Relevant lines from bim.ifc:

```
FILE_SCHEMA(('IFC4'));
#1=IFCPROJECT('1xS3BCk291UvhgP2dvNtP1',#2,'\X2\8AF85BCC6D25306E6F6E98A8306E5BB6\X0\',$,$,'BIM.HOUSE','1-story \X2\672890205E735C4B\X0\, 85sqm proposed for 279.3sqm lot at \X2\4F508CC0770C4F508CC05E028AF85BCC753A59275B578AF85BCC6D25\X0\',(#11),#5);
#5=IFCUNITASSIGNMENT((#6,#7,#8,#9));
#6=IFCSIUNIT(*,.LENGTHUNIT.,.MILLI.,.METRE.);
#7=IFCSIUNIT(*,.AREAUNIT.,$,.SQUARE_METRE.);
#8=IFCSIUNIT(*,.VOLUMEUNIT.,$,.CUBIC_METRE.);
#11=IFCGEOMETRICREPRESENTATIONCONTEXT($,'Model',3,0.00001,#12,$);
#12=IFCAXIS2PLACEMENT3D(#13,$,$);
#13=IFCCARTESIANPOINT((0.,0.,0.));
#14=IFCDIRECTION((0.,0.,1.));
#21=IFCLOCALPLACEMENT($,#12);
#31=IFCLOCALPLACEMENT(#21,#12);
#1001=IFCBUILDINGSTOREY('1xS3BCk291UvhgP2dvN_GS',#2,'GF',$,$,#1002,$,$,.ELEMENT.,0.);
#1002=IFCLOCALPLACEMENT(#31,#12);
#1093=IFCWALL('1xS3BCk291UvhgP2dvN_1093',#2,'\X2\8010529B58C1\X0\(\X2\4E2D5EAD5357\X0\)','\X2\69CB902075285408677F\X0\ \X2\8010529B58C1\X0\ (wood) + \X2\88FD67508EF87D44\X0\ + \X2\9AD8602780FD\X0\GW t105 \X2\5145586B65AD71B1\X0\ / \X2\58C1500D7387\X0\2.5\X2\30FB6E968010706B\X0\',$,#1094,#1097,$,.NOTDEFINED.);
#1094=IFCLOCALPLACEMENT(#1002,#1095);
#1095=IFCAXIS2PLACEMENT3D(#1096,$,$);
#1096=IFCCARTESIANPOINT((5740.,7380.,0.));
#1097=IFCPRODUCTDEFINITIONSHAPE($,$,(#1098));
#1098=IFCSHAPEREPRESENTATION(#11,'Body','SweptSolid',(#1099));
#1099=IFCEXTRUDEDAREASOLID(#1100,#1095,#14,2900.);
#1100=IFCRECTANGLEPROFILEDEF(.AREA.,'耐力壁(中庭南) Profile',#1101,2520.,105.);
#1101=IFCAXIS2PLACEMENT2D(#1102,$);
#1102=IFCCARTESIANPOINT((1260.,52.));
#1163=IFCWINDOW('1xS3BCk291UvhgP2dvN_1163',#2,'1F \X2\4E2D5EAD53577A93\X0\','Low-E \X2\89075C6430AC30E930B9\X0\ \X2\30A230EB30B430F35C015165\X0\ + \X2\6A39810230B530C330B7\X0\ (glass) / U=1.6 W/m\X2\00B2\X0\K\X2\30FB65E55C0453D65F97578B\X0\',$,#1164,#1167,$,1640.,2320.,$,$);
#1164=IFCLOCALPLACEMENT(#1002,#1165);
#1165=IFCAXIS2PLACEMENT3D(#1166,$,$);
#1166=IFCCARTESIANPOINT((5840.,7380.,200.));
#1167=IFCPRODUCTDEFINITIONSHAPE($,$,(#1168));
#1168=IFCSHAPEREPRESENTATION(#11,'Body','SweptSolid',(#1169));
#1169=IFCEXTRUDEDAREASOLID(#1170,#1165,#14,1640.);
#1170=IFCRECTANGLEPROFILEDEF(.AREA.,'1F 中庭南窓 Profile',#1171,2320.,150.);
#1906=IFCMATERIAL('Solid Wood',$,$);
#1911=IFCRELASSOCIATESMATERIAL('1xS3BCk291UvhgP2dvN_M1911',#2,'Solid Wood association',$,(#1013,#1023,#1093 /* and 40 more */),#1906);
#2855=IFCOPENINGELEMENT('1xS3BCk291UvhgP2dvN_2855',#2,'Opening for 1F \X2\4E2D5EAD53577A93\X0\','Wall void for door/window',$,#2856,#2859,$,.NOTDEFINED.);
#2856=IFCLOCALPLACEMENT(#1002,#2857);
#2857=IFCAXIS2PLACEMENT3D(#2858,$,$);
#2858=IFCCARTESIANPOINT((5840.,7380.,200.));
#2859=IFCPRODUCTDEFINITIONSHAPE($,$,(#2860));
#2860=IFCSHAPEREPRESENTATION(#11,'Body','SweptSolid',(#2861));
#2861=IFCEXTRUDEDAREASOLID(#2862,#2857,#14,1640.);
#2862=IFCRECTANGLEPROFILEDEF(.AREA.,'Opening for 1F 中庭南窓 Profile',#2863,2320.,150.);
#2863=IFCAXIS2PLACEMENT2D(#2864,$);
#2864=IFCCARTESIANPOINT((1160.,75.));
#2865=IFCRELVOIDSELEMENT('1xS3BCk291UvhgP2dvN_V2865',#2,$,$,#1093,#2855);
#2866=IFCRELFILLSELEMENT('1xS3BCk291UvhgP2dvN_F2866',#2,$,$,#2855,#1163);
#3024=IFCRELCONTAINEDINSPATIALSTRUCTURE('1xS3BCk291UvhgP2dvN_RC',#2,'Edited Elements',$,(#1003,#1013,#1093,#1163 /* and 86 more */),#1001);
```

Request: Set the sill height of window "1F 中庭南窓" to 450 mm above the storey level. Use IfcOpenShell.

```python
import numpy as np
import ifcopenshell
import ifcopenshell.api.geometry
import ifcopenshell.geom
import ifcopenshell.util.element
import ifcopenshell.util.placement
import ifcopenshell.util.shape
import ifcopenshell.util.unit

model = ifcopenshell.open("bim.ifc")
unit_scale = ifcopenshell.util.unit.calculate_unit_scale(model)

window = model.by_guid("1xS3BCk291UvhgP2dvN_1163")
opening = window.FillsVoids[0].RelatingOpeningElement
storey = ifcopenshell.util.element.get_container(window, ifc_class="IfcBuildingStorey")
level = ifcopenshell.util.placement.get_local_placement(storey.ObjectPlacement)[2, 3]

# The opening's origin need not be at the sill, so measure its lowest point.
shape = ifcopenshell.geom.create_shape(ifcopenshell.geom.settings(), opening)
bottom = ifcopenshell.util.shape.get_shape_bottom_elevation(shape, shape.geometry) / unit_scale
dz = level + 0.45 / unit_scale - bottom

shift = np.array([0.0, 0.0, dz])
# The window is not placed relative to its opening, so move both.
for product in (opening, window):
    matrix = ifcopenshell.util.placement.get_local_placement(product.ObjectPlacement)
    matrix[:3, 3] += shift
    ifcopenshell.api.geometry.edit_object_placement(model, product=product, matrix=matrix, is_si=False)

print(f"moved by {dz * unit_scale:+.3f} m")

model.write("bim_updated.ifc")
```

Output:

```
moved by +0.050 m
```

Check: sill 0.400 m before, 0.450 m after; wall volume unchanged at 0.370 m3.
